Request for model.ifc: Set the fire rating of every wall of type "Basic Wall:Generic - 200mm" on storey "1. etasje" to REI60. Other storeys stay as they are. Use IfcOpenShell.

First a look at what the model holds.

```python
import ifcopenshell
import ifcopenshell.util.element

model = ifcopenshell.open("model.ifc")
print(model.schema)
storey = next(s for s in model.by_type("IfcBuildingStorey") if s.Name == "1. etasje")
walls = [e for e in ifcopenshell.util.element.get_decomposition(storey) if e.is_a("IfcWall")]
seen = {}
for e in walls:
    element_type = ifcopenshell.util.element.get_type(e)
    key = (element_type.Name if element_type != e and element_type else None, ifcopenshell.util.element.get_pset(e, "Pset_WallCommon", "FireRating"))
    seen[key] = seen.get(key, 0) + 1
for (name, value), count in sorted(seen.items(), key=str):
    print(count, "x", name, "|", value)
```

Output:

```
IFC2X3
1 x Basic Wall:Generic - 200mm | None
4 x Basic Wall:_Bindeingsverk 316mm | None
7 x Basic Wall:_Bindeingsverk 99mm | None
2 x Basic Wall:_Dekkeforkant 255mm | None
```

```python
import ifcopenshell
import ifcopenshell.api.pset
import ifcopenshell.util.element

model = ifcopenshell.open("model.ifc")

storey = next(s for s in model.by_type("IfcBuildingStorey") if s.Name == "1. etasje")
walls = [e for e in ifcopenshell.util.element.get_decomposition(storey) if e.is_a("IfcWall")]

count = 0
for e in walls:
    element_type = ifcopenshell.util.element.get_type(e)
    if element_type in (None, e) or element_type.Name != "Basic Wall:Generic - 200mm":
        continue
    # add_pset returns the element's existing set when there is one.
    pset = ifcopenshell.api.pset.add_pset(model, product=e, name="Pset_WallCommon")
    ifcopenshell.api.pset.edit_pset(model, pset=pset, properties={"FireRating": "REI60"})
    count += 1

print(count, "walls updated")

model.write("model_rev.ifc")
```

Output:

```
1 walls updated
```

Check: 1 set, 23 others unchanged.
